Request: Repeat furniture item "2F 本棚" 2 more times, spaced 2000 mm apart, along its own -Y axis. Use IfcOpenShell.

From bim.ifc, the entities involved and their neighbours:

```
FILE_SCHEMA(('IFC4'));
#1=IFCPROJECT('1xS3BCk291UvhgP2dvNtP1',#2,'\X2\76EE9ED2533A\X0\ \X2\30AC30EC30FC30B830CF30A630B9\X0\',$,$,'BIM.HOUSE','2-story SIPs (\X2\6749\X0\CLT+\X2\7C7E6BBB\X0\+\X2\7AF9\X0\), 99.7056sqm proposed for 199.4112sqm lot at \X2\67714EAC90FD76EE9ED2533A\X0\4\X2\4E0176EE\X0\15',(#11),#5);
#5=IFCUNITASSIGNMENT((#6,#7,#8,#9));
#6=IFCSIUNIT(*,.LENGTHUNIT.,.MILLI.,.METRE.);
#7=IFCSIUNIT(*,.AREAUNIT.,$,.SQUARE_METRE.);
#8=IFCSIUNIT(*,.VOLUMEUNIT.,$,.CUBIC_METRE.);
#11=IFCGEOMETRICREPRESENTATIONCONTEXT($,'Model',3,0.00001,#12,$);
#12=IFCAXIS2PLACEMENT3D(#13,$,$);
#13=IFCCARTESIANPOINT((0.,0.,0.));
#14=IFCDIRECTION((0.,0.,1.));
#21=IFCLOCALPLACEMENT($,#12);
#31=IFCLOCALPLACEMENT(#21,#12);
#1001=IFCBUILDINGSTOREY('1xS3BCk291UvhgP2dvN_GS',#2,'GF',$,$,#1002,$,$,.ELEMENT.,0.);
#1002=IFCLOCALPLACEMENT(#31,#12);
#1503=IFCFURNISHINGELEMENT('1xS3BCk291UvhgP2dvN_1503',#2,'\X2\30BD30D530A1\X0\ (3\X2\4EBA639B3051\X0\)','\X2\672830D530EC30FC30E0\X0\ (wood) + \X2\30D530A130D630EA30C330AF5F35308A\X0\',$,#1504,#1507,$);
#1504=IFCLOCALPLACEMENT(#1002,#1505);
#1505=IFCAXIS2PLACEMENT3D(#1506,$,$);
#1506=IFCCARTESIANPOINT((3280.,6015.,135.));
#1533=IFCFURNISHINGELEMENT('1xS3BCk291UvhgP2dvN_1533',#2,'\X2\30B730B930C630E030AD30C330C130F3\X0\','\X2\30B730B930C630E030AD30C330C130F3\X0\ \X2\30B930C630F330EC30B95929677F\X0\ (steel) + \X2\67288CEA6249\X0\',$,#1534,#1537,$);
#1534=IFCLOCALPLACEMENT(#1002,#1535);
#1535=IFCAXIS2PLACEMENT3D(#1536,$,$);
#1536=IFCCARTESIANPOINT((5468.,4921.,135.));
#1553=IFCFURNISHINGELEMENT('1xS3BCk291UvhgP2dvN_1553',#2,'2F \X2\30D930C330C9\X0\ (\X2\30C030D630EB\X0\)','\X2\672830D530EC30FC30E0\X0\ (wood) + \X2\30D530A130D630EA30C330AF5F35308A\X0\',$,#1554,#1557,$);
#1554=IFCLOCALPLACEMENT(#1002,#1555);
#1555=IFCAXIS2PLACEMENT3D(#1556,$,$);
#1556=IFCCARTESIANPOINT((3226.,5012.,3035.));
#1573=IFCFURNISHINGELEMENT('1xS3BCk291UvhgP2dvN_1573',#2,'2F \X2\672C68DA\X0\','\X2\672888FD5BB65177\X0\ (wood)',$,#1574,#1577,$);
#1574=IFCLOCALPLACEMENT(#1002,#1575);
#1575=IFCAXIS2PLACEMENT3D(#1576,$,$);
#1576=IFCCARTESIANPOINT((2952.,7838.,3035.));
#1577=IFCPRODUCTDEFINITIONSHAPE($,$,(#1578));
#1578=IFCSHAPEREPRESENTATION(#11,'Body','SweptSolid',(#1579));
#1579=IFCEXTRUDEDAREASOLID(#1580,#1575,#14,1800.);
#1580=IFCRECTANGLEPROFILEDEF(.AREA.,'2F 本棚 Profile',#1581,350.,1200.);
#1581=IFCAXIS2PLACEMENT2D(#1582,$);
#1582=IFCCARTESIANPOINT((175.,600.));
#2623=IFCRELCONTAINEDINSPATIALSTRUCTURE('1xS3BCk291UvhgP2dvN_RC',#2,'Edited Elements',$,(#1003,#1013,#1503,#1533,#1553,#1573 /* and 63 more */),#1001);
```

```python
import ifcopenshell
import ifcopenshell.api.geometry
import ifcopenshell.api.root
import ifcopenshell.util.element
import ifcopenshell.util.placement
import ifcopenshell.util.unit

model = ifcopenshell.open("bim.ifc")
unit_scale = ifcopenshell.util.unit.calculate_unit_scale(model)


def reuse_history(source, copy):
    """copy_class also copies each property set's owner history, people and application; keep the originals."""
    for rel in copy.IsDefinedBy:
        if rel.is_a("IfcRelDefinesByProperties") and (history := rel.RelatingPropertyDefinition.OwnerHistory):
            rel.RelatingPropertyDefinition.OwnerHistory = source.OwnerHistory
            ifcopenshell.util.element.remove_deep2(model, history)


source = model.by_id(1573)
base = ifcopenshell.util.placement.get_local_placement(source.ObjectPlacement)
step = -base[:3, 1] * 2 / unit_scale

for i in range(1, 3):
    copy = ifcopenshell.api.root.copy_class(model, product=source)
    copy.Representation = ifcopenshell.util.element.copy_deep(
        model, source.Representation, exclude=["IfcGeometricRepresentationContext", "IfcRepresentationMap"]
    )
    reuse_history(source, copy)
    matrix = base.copy()
    matrix[:3, 3] += i * step
    print("added at", matrix[:3, 3].round(3) + 0.0)
    ifcopenshell.api.geometry.edit_object_placement(model, product=copy, matrix=matrix, is_si=False)

model.write("bim_rev.ifc")
```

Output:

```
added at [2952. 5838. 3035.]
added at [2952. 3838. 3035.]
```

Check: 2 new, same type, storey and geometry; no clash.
